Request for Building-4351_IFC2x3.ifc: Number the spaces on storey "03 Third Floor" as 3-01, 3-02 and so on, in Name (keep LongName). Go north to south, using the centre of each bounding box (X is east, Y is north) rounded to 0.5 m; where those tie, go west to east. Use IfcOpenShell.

First a look at what the model holds.

```python
import ifcopenshell
import ifcopenshell.util.element
import ifcopenshell.util.placement

model = ifcopenshell.open("Building-4351_IFC2x3.ifc")
print(model.schema)
storey = next(s for s in model.by_type("IfcBuildingStorey") if s.Name == "03 Third Floor")
spaces = [e for e in ifcopenshell.util.element.get_decomposition(storey) if e.is_a("IfcSpace")]
for e in sorted(spaces, key=lambda e: e.id()):
    origin = ifcopenshell.util.placement.get_local_placement(e.ObjectPlacement)[:3, 3]
    print(e.id(), e.Name, e.LongName, origin.round(2) + 0.0, sep=" | ")
```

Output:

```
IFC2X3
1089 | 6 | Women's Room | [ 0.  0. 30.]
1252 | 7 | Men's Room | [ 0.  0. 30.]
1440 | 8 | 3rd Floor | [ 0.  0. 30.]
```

```python
import ifcopenshell
import ifcopenshell.geom
import ifcopenshell.util.element
import ifcopenshell.util.shape

model = ifcopenshell.open("Building-4351_IFC2x3.ifc")
settings = ifcopenshell.geom.settings()
settings.set("use-world-coords", True)


def centre(element):
    shape = ifcopenshell.geom.create_shape(settings, element)
    return ifcopenshell.util.shape.get_bbox_centroid(shape.geometry)


storey = next(s for s in model.by_type("IfcBuildingStorey") if s.Name == "03 Third Floor")
spaces = [e for e in ifcopenshell.util.element.get_decomposition(storey) if e.is_a("IfcSpace")]

# Insertion points can sit at a corner or the storey origin, so sort by the geometry (in metres).
centres = {e: centre(e) for e in spaces}
spaces.sort(key=lambda e: (-round(centres[e][1] / 0.5), centres[e][0]))

for i, e in enumerate(spaces, start=1):
    number = f"3-{i:02d}"
    e.Name = number
    print(e.id(), number)

model.write("Building-4351_IFC2x3_edited.ifc")
```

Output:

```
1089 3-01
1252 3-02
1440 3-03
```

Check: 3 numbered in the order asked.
